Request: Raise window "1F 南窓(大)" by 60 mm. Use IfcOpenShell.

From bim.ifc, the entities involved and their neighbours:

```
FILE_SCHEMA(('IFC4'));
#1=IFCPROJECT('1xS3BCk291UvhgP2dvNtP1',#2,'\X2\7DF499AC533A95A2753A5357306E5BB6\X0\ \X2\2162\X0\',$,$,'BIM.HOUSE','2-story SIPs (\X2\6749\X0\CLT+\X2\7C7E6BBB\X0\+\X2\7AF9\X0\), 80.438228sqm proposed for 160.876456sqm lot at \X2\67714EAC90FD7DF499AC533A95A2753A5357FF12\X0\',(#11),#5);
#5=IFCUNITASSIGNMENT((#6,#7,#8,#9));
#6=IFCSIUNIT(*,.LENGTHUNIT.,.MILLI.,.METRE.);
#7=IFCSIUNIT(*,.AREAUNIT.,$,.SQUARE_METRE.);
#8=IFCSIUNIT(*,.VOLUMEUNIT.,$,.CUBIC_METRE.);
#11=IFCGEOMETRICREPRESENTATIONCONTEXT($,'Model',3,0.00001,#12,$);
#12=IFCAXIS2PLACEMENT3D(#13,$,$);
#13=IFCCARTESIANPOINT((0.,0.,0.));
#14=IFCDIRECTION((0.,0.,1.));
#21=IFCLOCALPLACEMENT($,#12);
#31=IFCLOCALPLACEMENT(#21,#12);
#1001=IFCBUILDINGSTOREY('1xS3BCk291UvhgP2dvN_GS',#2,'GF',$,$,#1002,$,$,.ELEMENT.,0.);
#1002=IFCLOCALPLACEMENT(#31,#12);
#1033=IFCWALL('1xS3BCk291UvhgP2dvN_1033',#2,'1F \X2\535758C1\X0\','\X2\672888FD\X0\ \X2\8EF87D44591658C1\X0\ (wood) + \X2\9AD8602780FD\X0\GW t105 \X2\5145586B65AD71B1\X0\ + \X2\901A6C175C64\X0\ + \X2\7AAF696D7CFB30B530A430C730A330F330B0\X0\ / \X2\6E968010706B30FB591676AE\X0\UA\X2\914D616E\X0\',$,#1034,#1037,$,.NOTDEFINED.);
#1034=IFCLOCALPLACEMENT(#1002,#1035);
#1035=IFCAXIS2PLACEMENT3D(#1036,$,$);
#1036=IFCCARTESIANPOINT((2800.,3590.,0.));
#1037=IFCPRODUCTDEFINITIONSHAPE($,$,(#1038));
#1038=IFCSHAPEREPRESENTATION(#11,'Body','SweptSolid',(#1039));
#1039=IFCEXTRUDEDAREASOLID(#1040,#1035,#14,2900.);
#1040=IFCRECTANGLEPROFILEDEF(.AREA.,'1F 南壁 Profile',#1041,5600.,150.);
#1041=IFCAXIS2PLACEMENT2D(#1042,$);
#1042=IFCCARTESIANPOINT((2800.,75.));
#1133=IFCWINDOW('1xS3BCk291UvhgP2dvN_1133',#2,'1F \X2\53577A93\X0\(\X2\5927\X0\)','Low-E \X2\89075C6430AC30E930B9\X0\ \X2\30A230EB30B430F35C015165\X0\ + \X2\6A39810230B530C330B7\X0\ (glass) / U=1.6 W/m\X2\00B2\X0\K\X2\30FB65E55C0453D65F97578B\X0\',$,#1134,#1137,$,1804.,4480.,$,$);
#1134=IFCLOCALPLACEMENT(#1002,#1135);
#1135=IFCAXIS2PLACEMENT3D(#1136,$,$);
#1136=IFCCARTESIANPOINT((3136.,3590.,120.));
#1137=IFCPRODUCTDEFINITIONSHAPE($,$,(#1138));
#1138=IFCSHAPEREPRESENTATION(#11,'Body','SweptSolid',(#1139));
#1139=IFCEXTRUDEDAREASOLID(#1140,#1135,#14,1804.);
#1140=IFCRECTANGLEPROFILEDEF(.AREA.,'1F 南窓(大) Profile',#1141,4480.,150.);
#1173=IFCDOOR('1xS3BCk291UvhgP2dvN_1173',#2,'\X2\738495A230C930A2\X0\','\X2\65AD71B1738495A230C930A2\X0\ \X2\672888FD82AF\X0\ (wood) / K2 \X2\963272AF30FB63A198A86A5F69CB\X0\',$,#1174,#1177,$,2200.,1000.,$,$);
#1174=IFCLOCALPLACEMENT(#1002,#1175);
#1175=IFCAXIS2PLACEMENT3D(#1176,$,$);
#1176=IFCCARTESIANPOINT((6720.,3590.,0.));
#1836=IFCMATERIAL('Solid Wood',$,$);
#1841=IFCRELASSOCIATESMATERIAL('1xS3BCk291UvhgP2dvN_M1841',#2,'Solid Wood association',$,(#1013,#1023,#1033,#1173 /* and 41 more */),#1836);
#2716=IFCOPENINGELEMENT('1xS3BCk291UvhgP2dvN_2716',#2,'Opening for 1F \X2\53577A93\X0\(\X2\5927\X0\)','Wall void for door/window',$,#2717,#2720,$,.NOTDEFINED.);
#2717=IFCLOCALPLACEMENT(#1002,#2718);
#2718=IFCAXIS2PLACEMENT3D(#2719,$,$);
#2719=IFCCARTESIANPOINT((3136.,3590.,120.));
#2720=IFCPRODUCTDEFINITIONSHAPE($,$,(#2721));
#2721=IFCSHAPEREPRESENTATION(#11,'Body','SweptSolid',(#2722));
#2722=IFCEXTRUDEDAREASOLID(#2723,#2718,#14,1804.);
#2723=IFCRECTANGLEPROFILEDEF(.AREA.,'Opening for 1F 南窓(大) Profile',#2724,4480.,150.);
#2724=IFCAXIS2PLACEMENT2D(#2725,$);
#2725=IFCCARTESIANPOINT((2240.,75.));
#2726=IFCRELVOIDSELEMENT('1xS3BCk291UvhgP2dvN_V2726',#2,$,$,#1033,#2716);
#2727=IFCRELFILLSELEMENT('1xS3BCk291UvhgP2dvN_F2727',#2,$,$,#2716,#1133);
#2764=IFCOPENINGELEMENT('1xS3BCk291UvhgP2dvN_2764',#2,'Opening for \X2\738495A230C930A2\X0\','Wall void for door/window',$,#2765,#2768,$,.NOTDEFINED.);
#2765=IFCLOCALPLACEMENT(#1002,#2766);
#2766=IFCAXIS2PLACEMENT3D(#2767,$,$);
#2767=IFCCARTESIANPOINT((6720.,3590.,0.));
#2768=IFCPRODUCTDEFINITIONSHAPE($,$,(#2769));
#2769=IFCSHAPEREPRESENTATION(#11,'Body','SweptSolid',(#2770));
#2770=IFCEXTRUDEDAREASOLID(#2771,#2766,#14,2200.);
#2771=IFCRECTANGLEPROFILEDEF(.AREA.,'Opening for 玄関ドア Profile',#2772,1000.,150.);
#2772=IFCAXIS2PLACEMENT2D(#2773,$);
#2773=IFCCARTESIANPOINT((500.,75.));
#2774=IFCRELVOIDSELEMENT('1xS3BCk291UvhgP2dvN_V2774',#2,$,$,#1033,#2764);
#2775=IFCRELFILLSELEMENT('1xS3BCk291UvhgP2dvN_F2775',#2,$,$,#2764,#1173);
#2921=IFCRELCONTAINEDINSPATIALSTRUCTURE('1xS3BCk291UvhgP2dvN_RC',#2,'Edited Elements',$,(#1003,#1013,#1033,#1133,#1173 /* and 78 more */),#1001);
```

```python
import numpy as np
import ifcopenshell
import ifcopenshell.api.geometry
import ifcopenshell.util.placement
import ifcopenshell.util.unit

model = ifcopenshell.open("bim.ifc")
unit_scale = ifcopenshell.util.unit.calculate_unit_scale(model)

window = model.by_guid("1xS3BCk291UvhgP2dvN_1133")
opening = window.FillsVoids[0].RelatingOpeningElement
dz = 0.06 / unit_scale

shift = np.array([0.0, 0.0, dz])
# The window is not placed relative to its opening, so move both.
for product in (opening, window):
    matrix = ifcopenshell.util.placement.get_local_placement(product.ObjectPlacement)
    matrix[:3, 3] += shift
    ifcopenshell.api.geometry.edit_object_placement(model, product=product, matrix=matrix, is_si=False)

print(f"moved by {dz * unit_scale:+.3f} m")

model.write("bim_updated.ifc")
```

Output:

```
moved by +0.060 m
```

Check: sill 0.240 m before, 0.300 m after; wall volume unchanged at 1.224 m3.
